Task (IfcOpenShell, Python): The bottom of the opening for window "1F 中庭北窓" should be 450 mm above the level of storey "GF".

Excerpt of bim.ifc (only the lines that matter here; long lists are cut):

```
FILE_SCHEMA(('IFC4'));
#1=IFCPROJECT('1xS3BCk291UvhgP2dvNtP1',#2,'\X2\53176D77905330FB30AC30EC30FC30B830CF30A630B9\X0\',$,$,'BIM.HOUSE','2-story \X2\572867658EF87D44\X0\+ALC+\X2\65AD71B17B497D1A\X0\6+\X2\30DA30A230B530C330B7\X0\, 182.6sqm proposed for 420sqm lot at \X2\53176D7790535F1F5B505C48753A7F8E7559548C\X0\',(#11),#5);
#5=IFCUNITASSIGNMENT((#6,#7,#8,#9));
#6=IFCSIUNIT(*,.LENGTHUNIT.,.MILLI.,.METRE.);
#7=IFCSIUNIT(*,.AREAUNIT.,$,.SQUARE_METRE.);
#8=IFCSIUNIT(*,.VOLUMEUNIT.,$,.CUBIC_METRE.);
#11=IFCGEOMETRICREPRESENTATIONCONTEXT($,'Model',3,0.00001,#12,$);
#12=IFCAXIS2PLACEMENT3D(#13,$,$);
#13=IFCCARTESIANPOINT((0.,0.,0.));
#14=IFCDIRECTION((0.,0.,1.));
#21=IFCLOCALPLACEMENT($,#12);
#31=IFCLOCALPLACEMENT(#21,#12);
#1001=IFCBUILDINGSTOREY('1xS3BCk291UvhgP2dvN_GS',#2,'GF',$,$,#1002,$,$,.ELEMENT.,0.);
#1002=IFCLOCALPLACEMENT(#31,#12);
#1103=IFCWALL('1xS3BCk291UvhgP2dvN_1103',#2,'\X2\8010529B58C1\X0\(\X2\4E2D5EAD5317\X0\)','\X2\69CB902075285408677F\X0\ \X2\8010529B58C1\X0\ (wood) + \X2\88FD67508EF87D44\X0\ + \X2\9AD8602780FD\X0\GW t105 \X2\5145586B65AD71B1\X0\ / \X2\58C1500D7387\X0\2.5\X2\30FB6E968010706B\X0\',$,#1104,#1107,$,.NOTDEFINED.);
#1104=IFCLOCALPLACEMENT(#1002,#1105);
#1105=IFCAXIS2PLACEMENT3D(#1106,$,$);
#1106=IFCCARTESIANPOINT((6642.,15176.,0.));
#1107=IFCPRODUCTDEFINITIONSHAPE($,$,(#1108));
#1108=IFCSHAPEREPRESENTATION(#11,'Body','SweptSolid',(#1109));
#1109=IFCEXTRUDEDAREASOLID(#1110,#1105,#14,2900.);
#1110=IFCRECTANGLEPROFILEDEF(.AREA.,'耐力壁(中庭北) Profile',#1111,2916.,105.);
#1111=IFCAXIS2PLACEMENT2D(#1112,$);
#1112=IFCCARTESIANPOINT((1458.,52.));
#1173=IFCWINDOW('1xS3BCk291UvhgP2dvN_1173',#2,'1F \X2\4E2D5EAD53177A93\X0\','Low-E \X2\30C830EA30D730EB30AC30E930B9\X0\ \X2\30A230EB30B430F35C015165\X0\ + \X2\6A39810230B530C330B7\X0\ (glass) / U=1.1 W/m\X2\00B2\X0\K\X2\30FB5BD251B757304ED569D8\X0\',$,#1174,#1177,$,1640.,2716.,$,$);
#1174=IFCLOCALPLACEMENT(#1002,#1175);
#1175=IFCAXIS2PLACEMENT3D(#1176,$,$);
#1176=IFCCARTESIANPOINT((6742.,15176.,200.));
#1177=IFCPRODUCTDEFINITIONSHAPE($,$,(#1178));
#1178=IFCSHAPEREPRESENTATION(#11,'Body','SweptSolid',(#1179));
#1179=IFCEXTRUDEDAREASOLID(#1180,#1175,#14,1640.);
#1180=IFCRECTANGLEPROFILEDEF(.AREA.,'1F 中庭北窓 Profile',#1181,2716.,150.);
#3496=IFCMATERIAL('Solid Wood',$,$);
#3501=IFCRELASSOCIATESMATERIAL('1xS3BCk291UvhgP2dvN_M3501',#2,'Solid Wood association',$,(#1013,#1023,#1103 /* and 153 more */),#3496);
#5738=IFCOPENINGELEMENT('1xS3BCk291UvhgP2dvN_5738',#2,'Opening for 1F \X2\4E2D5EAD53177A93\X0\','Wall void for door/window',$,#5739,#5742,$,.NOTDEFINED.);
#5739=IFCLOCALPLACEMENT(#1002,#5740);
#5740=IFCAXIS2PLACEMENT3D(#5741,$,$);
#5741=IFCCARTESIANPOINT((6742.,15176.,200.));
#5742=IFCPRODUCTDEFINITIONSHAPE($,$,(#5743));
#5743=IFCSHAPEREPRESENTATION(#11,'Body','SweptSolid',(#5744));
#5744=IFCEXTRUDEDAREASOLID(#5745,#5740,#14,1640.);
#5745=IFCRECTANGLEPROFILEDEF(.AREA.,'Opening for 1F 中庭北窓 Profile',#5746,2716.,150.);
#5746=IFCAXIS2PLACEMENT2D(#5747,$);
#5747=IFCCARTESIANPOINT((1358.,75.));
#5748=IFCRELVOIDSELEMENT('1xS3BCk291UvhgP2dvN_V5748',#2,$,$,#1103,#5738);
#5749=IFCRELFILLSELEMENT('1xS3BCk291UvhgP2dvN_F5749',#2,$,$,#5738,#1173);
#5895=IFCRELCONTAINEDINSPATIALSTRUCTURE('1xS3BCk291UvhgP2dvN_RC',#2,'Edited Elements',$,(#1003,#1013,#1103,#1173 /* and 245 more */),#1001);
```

```python
import numpy as np
import ifcopenshell
import ifcopenshell.api.geometry
import ifcopenshell.geom
import ifcopenshell.util.element
import ifcopenshell.util.placement
import ifcopenshell.util.shape
import ifcopenshell.util.unit

model = ifcopenshell.open("bim.ifc")
unit_scale = ifcopenshell.util.unit.calculate_unit_scale(model)

window = model.by_guid("1xS3BCk291UvhgP2dvN_1173")
opening = window.FillsVoids[0].RelatingOpeningElement
storey = ifcopenshell.util.element.get_container(window, ifc_class="IfcBuildingStorey")
level = ifcopenshell.util.placement.get_local_placement(storey.ObjectPlacement)[2, 3]

# The opening's origin need not be at the sill, so measure its lowest point.
shape = ifcopenshell.geom.create_shape(ifcopenshell.geom.settings(), opening)
bottom = ifcopenshell.util.shape.get_shape_bottom_elevation(shape, shape.geometry) / unit_scale
dz = level + 450.0 - bottom

shift = np.array([0.0, 0.0, dz])
# The window is not placed relative to its opening, so move both.
for product in (opening, window):
    matrix = ifcopenshell.util.placement.get_local_placement(product.ObjectPlacement)
    matrix[:3, 3] += shift
    ifcopenshell.api.geometry.edit_object_placement(model, product=product, matrix=matrix, is_si=False)

print(f"moved by {dz * unit_scale:+.3f} m")

model.write("bim-out.ifc")
```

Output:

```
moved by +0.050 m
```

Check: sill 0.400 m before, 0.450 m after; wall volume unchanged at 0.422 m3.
